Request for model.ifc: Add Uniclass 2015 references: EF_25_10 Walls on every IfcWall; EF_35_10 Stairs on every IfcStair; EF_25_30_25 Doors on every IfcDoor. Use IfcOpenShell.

First a look at what the model holds.

```python
import ifcopenshell

model = ifcopenshell.open("model.ifc")
print(model.schema)
print("classifications:", [c.Name for c in model.by_type("IfcClassification")])
for ifc_class in ("IfcDoor", "IfcRoof", "IfcStair", "IfcWall", "IfcWindow"):
    print(ifc_class, len(model.by_type(ifc_class)))
```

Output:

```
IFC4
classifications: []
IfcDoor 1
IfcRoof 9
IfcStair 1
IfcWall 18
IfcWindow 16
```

```python
import ifcopenshell
import ifcopenshell.api.classification

model = ifcopenshell.open("model.ifc")

system = ifcopenshell.api.classification.add_classification(model, classification="Uniclass 2015")

codes = {
    "IfcWall": ("EF_25_10", "Walls"),
    "IfcStair": ("EF_35_10", "Stairs"),
    "IfcDoor": ("EF_25_30_25", "Doors"),
}
for ifc_class, (code, name) in codes.items():
    products = model.by_type(ifc_class)
    ifcopenshell.api.classification.add_reference(
        model, products=products, classification=system, identification=code, name=name
    )
    print(code, len(products))

model.write("model_rev.ifc")
```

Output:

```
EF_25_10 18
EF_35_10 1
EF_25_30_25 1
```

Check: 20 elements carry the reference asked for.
